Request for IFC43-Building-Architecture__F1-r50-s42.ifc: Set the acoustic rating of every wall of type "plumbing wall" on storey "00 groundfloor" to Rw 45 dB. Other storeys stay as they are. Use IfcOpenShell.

First a look at what the model holds.

```python
import ifcopenshell
import ifcopenshell.util.element

model = ifcopenshell.open("IFC43-Building-Architecture__F1-r50-s42.ifc")
print(model.schema)
storey = next(s for s in model.by_type("IfcBuildingStorey") if s.Name == "00 groundfloor")
walls = [e for e in ifcopenshell.util.element.get_decomposition(storey) if e.is_a("IfcWall")]
seen = {}
for e in walls:
    element_type = ifcopenshell.util.element.get_type(e)
    key = (element_type.Name if element_type != e and element_type else None, ifcopenshell.util.element.get_pset(e, "Pset_WallCommon", "AcousticRating"))
    seen[key] = seen.get(key, 0) + 1
for (name, value), count in sorted(seen.items(), key=str):
    print(count, "x", name, "|", value)
```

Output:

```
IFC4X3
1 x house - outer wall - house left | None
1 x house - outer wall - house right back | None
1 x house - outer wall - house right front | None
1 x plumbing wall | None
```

```python
import ifcopenshell
import ifcopenshell.api.pset
import ifcopenshell.util.element

model = ifcopenshell.open("IFC43-Building-Architecture__F1-r50-s42.ifc")

storey = next(s for s in model.by_type("IfcBuildingStorey") if s.Name == "00 groundfloor")
walls = [e for e in ifcopenshell.util.element.get_decomposition(storey) if e.is_a("IfcWall")]

count = 0
for e in walls:
    element_type = ifcopenshell.util.element.get_type(e)
    if element_type in (None, e) or element_type.Name != "plumbing wall":
        continue
    # add_pset returns the element's existing set when there is one.
    pset = ifcopenshell.api.pset.add_pset(model, product=e, name="Pset_WallCommon")
    ifcopenshell.api.pset.edit_pset(model, pset=pset, properties={"AcousticRating": "Rw 45 dB"})
    count += 1

print(count, "walls updated")

model.write("IFC43-Building-Architecture__F1-r50-s42_v2.ifc")
```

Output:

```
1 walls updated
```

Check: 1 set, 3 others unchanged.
